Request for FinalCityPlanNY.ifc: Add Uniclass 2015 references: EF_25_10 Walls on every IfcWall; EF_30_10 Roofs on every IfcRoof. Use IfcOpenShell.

First a look at what the model holds.

```python
import ifcopenshell

model = ifcopenshell.open("FinalCityPlanNY.ifc")
print(model.schema)
print("classifications:", [c.Name for c in model.by_type("IfcClassification")])
for ifc_class in ("IfcDoor", "IfcRoof", "IfcStair", "IfcWall", "IfcWindow"):
    print(ifc_class, len(model.by_type(ifc_class)))
```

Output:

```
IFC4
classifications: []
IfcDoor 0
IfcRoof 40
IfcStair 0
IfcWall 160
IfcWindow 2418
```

```python
import ifcopenshell
import ifcopenshell.api.classification

model = ifcopenshell.open("FinalCityPlanNY.ifc")

system = ifcopenshell.api.classification.add_classification(model, classification="Uniclass 2015")

codes = {
    "IfcWall": ("EF_25_10", "Walls"),
    "IfcRoof": ("EF_30_10", "Roofs"),
}
for ifc_class, (code, name) in codes.items():
    products = model.by_type(ifc_class)
    ifcopenshell.api.classification.add_reference(
        model, products=products, classification=system, identification=code, name=name
    )
    print(code, len(products))

model.write("FinalCityPlanNY-out.ifc")
```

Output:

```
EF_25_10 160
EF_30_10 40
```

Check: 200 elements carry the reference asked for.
